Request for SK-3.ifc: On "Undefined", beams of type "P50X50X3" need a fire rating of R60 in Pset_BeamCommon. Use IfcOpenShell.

First a look at what the model holds.

```python
import ifcopenshell
import ifcopenshell.util.element

model = ifcopenshell.open("SK-3.ifc")
print(model.schema)
storey = next(s for s in model.by_type("IfcBuildingStorey") if s.Name == "Undefined")
beams = [e for e in ifcopenshell.util.element.get_decomposition(storey) if e.is_a("IfcBeam")]
seen = {}
for e in beams:
    element_type = ifcopenshell.util.element.get_type(e)
    key = (element_type.Name if element_type != e and element_type else None, ifcopenshell.util.element.get_pset(e, "Pset_BeamCommon", "FireRating"))
    seen[key] = seen.get(key, 0) + 1
for (name, value), count in sorted(seen.items(), key=str):
    print(count, "x", name, "|", value)
```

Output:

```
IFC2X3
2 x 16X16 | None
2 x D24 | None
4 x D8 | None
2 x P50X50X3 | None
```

```python
import ifcopenshell
import ifcopenshell.api.pset
import ifcopenshell.util.element

model = ifcopenshell.open("SK-3.ifc")

storey = next(s for s in model.by_type("IfcBuildingStorey") if s.Name == "Undefined")
beams = [e for e in ifcopenshell.util.element.get_decomposition(storey) if e.is_a("IfcBeam")]

count = 0
for e in beams:
    element_type = ifcopenshell.util.element.get_type(e)
    if element_type in (None, e) or element_type.Name != "P50X50X3":
        continue
    found = ifcopenshell.util.element.get_pset(e, "Pset_BeamCommon", should_inherit=False)
    if found:
        pset = model.by_id(found["id"])
        if len(ifcopenshell.util.element.get_elements_by_pset(pset)) > 1:
            pset = ifcopenshell.api.pset.unshare_pset(model, products=[e], pset=pset)[0]
    else:
        pset = ifcopenshell.api.pset.add_pset(model, product=e, name="Pset_BeamCommon")
    ifcopenshell.api.pset.edit_pset(model, pset=pset, properties={"FireRating": "R60"})
    count += 1

print(count, "beams updated")

model.write("SK-3_v2.ifc")
```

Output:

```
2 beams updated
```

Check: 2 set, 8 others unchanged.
